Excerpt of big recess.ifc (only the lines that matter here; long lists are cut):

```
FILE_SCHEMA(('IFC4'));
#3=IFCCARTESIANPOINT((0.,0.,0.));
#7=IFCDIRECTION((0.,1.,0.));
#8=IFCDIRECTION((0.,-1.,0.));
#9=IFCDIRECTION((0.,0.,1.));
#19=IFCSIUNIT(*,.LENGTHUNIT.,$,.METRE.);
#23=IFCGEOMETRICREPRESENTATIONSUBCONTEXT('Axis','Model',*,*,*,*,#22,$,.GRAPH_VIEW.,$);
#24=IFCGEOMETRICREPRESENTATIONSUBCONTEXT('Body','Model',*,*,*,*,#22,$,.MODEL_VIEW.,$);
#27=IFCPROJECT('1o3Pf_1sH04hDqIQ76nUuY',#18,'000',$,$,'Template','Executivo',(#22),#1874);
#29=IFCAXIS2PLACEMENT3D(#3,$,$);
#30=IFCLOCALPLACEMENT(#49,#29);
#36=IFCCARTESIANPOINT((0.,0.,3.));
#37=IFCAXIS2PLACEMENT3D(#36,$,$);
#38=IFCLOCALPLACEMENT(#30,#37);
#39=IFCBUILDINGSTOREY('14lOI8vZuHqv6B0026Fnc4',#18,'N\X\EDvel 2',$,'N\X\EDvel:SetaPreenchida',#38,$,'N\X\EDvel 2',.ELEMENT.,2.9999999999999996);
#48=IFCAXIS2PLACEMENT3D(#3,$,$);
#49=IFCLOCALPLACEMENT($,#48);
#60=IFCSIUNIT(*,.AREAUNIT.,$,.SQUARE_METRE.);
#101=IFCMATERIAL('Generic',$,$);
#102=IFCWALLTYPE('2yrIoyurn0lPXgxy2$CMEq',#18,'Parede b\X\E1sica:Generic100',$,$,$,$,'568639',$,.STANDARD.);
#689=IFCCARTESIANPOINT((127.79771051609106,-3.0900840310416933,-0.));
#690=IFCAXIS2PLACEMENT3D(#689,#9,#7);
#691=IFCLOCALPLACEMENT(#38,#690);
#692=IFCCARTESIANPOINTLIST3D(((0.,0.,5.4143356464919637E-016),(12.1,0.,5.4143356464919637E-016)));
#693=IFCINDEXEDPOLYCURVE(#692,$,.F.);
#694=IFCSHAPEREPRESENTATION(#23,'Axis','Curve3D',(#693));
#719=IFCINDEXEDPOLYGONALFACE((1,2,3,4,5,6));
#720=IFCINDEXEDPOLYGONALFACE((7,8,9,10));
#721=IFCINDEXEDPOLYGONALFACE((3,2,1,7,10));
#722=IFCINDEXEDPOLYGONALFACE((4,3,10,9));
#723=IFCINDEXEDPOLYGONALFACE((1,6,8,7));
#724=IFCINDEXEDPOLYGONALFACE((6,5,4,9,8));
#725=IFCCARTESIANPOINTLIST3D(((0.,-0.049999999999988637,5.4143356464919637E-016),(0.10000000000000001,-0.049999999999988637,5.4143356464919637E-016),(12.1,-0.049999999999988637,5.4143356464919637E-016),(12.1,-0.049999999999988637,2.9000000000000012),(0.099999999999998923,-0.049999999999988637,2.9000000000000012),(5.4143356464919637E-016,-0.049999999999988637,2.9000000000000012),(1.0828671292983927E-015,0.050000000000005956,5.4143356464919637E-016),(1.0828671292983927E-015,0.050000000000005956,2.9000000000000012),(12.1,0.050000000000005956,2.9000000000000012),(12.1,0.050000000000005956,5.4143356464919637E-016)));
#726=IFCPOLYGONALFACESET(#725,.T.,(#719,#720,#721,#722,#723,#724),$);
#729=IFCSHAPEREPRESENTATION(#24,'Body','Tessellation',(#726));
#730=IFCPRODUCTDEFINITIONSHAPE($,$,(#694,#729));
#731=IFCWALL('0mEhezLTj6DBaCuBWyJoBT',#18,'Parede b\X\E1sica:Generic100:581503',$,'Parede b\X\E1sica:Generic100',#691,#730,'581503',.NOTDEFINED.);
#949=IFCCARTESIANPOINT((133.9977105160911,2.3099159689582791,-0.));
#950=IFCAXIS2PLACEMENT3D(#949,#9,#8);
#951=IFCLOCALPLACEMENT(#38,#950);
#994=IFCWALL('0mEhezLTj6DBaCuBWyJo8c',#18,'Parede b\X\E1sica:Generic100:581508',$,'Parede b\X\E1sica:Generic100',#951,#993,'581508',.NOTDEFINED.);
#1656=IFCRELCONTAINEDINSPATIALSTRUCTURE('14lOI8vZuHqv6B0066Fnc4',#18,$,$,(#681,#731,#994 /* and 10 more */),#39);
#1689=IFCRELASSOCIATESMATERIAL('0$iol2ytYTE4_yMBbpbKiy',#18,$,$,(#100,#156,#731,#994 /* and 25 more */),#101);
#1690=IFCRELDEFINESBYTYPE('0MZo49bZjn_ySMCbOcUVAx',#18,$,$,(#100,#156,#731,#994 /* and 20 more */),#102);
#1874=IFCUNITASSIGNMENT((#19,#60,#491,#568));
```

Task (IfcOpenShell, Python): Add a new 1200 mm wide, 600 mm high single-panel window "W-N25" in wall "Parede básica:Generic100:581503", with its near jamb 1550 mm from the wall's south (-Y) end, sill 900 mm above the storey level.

```python
import numpy as np
import ifcopenshell
import ifcopenshell.api.feature
import ifcopenshell.api.geometry
import ifcopenshell.api.root
import ifcopenshell.api.spatial
import ifcopenshell.geom
import ifcopenshell.util.element
import ifcopenshell.util.placement
import ifcopenshell.util.representation
import ifcopenshell.util.shape
import ifcopenshell.util.unit

model = ifcopenshell.open("big recess.ifc")
unit_scale = ifcopenshell.util.unit.calculate_unit_scale(model)
settings = ifcopenshell.geom.settings()


def volume(element):
    """Net volume in cubic metres, openings subtracted."""
    shape = ifcopenshell.geom.create_shape(settings, element)
    return ifcopenshell.util.shape.get_volume(shape.geometry)


wall = model.by_guid("0mEhezLTj6DBaCuBWyJoBT")
storey = ifcopenshell.util.element.get_container(wall, ifc_class="IfcBuildingStorey")
context = ifcopenshell.util.representation.get_context(model, "Model", "Body", "MODEL_VIEW")
before = volume(wall)

width, height, from_end, sill = 1.2, 0.6, 1.55, 0.9  # metres

# The wall runs along its own X axis, and the end named is its -X end.
wall_shape = ifcopenshell.geom.create_shape(settings, wall)
x, y, z = ifcopenshell.util.shape.get_vertices(wall_shape.geometry).T
start = x.min() + from_end
face, thickness = float(y.min()), float(y.max() - y.min())
wall_matrix = ifcopenshell.util.placement.get_local_placement(wall.ObjectPlacement)
level = ifcopenshell.util.placement.get_local_placement(storey.ObjectPlacement)[2, 3]


def in_wall(x, y):
    """Placement at x, y metres in the wall's axes, at sill height."""
    matrix = wall_matrix.copy()
    matrix[:, 3] = wall_matrix @ np.array([x / unit_scale, y / unit_scale, 0.0, 1.0])
    matrix[2, 3] = level + sill / unit_scale
    return matrix


# Opening: a box that overshoots both wall faces by 50 mm.
opening = ifcopenshell.api.root.create_entity(model, ifc_class="IfcOpeningElement", predefined_type="OPENING")
box = ifcopenshell.api.geometry.add_wall_representation(
    model, context=context, length=width, height=height, thickness=thickness + 0.1
)
ifcopenshell.api.geometry.assign_representation(model, product=opening, representation=box)
ifcopenshell.api.geometry.edit_object_placement(model, product=opening, matrix=in_wall(start, face - 0.05), is_si=False)
ifcopenshell.api.feature.add_feature(model, feature=opening, element=wall)

window = ifcopenshell.api.root.create_entity(model, ifc_class="IfcWindow", name="W-N25", predefined_type="WINDOW")
window.OverallWidth, window.OverallHeight = width / unit_scale, height / unit_scale
window.PartitioningType = "SINGLE_PANEL"
body = ifcopenshell.api.geometry.add_window_representation(
    model,
    context=context,
    overall_width=window.OverallWidth,
    overall_height=window.OverallHeight,
    partition_type="SINGLE_PANEL",
)
ifcopenshell.api.geometry.assign_representation(model, product=window, representation=body)
ifcopenshell.api.spatial.assign_container(model, products=[window], relating_structure=storey)
ifcopenshell.api.feature.add_filling(model, opening=opening, element=window)

# Centre the window in the wall's thickness.
ifcopenshell.api.geometry.edit_object_placement(model, product=window, matrix=in_wall(start, face), is_si=False)
window_shape = ifcopenshell.geom.create_shape(settings, window)
depth = ifcopenshell.util.shape.get_vertices(window_shape.geometry)[:, 1]
offset = face + thickness / 2 - (depth.min() + depth.max()) / 2
ifcopenshell.api.geometry.edit_object_placement(model, product=window, matrix=in_wall(start, offset), is_si=False)

after = volume(wall)

print(f"wall volume {before:.3f} -> {after:.3f} m3")

model.write("big recess_updated.ifc")
```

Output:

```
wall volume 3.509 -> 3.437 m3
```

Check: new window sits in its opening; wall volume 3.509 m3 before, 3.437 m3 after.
